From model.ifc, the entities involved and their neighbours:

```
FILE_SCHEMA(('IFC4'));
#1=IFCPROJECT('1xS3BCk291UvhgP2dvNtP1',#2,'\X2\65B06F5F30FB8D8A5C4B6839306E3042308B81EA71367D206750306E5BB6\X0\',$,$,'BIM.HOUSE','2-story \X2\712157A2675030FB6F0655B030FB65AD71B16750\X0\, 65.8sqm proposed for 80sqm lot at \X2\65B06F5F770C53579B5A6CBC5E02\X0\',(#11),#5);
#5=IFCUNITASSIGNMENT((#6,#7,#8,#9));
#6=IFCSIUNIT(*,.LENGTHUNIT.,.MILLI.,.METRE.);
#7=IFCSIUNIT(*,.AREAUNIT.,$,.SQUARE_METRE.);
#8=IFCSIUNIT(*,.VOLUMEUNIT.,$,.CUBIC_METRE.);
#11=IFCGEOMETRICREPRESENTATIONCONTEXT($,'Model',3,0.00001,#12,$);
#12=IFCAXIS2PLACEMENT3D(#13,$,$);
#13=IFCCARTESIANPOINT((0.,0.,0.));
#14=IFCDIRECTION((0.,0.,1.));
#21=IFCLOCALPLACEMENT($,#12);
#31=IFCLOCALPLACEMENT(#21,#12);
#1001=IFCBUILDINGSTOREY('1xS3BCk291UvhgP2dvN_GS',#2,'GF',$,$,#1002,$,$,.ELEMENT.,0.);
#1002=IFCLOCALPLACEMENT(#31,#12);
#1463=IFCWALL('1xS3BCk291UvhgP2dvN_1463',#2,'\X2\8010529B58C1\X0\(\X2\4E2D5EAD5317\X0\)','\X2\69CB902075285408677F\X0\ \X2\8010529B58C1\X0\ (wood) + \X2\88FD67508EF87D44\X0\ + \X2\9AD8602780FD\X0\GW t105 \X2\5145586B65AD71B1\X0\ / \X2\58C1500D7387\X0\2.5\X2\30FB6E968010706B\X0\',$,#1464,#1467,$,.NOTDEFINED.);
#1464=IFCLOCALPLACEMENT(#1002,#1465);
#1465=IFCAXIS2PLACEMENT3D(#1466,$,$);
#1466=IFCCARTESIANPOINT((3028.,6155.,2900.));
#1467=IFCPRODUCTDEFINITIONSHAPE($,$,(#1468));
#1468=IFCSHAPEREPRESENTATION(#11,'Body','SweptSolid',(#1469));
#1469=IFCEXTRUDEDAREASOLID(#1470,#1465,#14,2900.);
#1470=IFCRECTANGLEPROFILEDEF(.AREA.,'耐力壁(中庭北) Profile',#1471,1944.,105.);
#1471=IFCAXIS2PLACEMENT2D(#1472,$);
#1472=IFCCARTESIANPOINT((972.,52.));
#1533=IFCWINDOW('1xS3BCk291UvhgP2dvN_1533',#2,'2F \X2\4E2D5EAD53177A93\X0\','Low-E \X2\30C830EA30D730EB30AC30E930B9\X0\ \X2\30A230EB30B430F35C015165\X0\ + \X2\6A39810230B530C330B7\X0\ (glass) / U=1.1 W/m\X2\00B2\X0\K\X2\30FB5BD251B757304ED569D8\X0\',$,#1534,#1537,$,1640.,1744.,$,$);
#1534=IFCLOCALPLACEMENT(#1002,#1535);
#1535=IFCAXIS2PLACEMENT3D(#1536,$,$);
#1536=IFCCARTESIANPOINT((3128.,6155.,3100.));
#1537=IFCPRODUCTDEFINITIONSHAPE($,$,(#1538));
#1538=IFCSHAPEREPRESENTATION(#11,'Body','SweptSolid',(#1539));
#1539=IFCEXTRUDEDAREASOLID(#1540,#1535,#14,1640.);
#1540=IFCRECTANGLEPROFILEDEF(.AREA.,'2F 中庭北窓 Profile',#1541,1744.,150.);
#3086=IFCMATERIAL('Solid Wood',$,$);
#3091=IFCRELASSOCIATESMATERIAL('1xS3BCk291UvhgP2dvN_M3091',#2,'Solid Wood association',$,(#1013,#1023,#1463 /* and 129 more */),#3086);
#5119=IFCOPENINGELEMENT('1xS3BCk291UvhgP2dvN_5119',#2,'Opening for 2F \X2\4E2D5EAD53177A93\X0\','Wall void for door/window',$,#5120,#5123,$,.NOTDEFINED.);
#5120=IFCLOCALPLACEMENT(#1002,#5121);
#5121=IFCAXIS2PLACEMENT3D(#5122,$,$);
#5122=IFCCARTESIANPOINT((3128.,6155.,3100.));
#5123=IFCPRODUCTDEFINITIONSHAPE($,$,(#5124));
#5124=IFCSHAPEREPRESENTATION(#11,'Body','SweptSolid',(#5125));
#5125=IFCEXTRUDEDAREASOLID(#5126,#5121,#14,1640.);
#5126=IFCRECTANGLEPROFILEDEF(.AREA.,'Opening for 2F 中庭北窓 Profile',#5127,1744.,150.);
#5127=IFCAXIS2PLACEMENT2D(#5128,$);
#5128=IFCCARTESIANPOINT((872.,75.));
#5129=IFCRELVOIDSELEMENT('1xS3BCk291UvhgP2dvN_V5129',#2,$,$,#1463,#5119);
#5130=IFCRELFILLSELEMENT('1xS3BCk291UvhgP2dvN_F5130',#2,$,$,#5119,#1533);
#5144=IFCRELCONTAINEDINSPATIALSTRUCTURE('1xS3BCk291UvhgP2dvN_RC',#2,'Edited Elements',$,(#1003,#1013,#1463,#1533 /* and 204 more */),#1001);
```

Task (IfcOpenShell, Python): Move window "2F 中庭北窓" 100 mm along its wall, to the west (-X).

```python
import ifcopenshell
import ifcopenshell.api.geometry
import ifcopenshell.util.placement
import ifcopenshell.util.unit

model = ifcopenshell.open("model.ifc")
unit_scale = ifcopenshell.util.unit.calculate_unit_scale(model)

window = model.by_guid("1xS3BCk291UvhgP2dvN_1533")
opening = window.FillsVoids[0].RelatingOpeningElement
wall = opening.VoidsElements[0].RelatingBuildingElement

wall_matrix = ifcopenshell.util.placement.get_local_placement(wall.ObjectPlacement)
shift = wall_matrix[:3, 0] * -0.1 / unit_scale
before = ifcopenshell.util.placement.get_local_placement(window.ObjectPlacement)[:3, 3].copy()

# The window is not placed relative to its opening, so move both.
for product in (opening, window):
    matrix = ifcopenshell.util.placement.get_local_placement(product.ObjectPlacement)
    matrix[:3, 3] += shift
    ifcopenshell.api.geometry.edit_object_placement(model, product=product, matrix=matrix, is_si=False)

after = ifcopenshell.util.placement.get_local_placement(window.ObjectPlacement)[:3, 3]
print("window moved by", (after - before).round(3) + 0.0)

model.write("model_v2.ifc")
```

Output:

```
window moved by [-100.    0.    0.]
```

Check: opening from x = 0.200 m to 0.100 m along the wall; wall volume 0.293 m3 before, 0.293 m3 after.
